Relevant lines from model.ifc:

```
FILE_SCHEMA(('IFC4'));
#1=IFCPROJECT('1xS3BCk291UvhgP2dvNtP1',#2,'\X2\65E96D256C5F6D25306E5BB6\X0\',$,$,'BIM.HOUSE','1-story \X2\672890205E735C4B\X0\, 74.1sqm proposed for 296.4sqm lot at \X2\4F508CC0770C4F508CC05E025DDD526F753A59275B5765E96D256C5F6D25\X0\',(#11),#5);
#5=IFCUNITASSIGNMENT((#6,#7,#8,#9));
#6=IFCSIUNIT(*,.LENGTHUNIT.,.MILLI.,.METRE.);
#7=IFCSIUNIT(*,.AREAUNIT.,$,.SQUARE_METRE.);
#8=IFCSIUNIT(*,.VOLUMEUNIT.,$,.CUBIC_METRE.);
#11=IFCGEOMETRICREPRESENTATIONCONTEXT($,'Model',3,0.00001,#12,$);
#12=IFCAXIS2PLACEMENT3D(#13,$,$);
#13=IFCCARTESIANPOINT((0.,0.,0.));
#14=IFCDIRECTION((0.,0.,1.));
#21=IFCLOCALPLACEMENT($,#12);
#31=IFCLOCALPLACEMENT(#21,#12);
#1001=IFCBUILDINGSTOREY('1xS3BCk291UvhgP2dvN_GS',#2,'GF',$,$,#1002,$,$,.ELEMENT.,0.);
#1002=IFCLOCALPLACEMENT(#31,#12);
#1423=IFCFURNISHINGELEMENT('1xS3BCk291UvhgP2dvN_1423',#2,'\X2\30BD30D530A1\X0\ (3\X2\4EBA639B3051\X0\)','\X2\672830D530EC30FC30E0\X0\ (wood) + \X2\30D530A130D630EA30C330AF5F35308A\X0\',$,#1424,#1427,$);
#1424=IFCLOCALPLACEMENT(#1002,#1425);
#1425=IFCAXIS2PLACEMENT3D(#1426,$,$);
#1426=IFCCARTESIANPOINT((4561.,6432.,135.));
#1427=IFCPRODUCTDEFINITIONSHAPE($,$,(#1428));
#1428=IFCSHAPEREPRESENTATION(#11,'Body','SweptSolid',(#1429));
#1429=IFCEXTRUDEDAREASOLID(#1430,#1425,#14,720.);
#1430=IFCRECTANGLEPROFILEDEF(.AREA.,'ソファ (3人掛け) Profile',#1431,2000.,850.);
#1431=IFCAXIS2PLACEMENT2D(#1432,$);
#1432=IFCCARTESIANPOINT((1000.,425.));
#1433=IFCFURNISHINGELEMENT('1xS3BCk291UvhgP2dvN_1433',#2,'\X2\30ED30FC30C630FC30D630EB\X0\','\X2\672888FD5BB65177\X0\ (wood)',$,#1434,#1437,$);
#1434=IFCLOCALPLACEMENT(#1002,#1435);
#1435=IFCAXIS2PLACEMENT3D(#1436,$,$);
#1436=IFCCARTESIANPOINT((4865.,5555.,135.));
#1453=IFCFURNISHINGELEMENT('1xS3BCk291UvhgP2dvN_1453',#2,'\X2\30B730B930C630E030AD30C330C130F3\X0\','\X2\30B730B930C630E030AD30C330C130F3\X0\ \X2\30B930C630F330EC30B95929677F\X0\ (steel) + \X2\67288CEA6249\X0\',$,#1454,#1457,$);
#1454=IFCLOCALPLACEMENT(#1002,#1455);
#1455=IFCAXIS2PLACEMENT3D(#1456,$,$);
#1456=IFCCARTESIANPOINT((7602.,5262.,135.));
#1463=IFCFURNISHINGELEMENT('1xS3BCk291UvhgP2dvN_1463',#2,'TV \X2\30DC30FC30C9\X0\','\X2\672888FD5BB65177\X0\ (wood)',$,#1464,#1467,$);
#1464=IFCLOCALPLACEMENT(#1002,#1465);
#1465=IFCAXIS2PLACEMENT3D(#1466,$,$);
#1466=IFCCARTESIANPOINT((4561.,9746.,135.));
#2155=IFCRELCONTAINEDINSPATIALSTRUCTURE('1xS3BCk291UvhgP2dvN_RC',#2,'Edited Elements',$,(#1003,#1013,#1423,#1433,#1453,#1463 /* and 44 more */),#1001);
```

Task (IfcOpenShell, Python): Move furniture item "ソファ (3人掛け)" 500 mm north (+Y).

```python
import ifcopenshell
import ifcopenshell.api.geometry
import ifcopenshell.util.placement
import ifcopenshell.util.unit

model = ifcopenshell.open("model.ifc")
unit_scale = ifcopenshell.util.unit.calculate_unit_scale(model)

item = model.by_id(1423)
matrix = ifcopenshell.util.placement.get_local_placement(item.ObjectPlacement)
matrix[1, 3] += 0.5 / unit_scale
ifcopenshell.api.geometry.edit_object_placement(model, product=item, matrix=matrix, is_si=False)

print(ifcopenshell.util.placement.get_local_placement(item.ObjectPlacement).round(3) + 0.0)

model.write("model_edited.ifc")
```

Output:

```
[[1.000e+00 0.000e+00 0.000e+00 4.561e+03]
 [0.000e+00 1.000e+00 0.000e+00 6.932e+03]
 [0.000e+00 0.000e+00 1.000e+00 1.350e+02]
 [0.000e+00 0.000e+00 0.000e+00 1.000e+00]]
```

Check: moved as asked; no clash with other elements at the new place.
